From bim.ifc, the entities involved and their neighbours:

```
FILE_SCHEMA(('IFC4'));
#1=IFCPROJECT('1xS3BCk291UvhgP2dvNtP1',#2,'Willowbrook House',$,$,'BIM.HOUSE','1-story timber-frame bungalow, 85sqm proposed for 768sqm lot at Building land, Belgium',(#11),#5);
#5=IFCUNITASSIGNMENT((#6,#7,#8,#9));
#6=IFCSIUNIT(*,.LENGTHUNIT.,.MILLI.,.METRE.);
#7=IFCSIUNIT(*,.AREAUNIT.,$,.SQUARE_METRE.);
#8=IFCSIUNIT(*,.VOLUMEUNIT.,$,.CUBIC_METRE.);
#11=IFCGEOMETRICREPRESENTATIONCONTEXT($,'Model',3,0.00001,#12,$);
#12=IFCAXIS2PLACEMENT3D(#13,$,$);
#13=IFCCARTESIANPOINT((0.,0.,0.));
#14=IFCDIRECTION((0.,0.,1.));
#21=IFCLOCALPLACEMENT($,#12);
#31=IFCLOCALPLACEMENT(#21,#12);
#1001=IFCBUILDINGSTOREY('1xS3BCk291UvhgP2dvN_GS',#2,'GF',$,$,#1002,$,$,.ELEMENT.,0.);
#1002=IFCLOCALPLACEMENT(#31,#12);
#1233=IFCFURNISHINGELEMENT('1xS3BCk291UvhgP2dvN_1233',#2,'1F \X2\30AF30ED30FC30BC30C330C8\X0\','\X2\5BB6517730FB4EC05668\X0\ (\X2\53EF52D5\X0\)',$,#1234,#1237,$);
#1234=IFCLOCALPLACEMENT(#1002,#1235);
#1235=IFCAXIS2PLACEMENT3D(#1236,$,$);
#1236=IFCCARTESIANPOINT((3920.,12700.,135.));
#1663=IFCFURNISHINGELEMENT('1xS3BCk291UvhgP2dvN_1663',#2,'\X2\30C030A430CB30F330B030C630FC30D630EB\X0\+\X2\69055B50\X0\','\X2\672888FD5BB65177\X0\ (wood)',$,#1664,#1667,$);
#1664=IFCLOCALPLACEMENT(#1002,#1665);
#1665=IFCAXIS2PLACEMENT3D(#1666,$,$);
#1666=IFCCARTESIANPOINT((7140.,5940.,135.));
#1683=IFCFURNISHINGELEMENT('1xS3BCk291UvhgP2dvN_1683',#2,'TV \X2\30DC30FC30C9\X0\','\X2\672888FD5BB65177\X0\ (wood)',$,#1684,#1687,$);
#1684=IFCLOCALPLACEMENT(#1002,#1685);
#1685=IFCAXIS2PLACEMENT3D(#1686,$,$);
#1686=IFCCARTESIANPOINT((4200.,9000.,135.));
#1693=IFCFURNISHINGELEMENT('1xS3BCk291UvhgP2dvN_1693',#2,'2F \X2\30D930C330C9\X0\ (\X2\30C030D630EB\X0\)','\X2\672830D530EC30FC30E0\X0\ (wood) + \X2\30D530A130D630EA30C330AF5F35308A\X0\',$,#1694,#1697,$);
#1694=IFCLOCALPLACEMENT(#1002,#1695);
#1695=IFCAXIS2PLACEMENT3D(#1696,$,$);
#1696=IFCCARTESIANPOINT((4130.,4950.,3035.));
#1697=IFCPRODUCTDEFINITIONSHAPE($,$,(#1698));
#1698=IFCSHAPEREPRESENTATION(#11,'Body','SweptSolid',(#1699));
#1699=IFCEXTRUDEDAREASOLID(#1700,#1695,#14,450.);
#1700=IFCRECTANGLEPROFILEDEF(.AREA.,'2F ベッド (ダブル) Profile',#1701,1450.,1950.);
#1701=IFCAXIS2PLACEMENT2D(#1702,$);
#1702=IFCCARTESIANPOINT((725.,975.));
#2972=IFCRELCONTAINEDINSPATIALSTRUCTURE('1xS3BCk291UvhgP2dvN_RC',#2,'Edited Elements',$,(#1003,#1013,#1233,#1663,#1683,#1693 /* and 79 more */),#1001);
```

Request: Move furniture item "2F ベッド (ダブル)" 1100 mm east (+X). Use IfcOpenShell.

```python
import ifcopenshell
import ifcopenshell.api.geometry
import ifcopenshell.util.placement

model = ifcopenshell.open("bim.ifc")

item = model.by_guid("1xS3BCk291UvhgP2dvN_1693")
matrix = ifcopenshell.util.placement.get_local_placement(item.ObjectPlacement)
matrix[0, 3] += 1100.0
ifcopenshell.api.geometry.edit_object_placement(model, product=item, matrix=matrix, is_si=False)

print(ifcopenshell.util.placement.get_local_placement(item.ObjectPlacement).round(3) + 0.0)

model.write("bim_rev.ifc")
```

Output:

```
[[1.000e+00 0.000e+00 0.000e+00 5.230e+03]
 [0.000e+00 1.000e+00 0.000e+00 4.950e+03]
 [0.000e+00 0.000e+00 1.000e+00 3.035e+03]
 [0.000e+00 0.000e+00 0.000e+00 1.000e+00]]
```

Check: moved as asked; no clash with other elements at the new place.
